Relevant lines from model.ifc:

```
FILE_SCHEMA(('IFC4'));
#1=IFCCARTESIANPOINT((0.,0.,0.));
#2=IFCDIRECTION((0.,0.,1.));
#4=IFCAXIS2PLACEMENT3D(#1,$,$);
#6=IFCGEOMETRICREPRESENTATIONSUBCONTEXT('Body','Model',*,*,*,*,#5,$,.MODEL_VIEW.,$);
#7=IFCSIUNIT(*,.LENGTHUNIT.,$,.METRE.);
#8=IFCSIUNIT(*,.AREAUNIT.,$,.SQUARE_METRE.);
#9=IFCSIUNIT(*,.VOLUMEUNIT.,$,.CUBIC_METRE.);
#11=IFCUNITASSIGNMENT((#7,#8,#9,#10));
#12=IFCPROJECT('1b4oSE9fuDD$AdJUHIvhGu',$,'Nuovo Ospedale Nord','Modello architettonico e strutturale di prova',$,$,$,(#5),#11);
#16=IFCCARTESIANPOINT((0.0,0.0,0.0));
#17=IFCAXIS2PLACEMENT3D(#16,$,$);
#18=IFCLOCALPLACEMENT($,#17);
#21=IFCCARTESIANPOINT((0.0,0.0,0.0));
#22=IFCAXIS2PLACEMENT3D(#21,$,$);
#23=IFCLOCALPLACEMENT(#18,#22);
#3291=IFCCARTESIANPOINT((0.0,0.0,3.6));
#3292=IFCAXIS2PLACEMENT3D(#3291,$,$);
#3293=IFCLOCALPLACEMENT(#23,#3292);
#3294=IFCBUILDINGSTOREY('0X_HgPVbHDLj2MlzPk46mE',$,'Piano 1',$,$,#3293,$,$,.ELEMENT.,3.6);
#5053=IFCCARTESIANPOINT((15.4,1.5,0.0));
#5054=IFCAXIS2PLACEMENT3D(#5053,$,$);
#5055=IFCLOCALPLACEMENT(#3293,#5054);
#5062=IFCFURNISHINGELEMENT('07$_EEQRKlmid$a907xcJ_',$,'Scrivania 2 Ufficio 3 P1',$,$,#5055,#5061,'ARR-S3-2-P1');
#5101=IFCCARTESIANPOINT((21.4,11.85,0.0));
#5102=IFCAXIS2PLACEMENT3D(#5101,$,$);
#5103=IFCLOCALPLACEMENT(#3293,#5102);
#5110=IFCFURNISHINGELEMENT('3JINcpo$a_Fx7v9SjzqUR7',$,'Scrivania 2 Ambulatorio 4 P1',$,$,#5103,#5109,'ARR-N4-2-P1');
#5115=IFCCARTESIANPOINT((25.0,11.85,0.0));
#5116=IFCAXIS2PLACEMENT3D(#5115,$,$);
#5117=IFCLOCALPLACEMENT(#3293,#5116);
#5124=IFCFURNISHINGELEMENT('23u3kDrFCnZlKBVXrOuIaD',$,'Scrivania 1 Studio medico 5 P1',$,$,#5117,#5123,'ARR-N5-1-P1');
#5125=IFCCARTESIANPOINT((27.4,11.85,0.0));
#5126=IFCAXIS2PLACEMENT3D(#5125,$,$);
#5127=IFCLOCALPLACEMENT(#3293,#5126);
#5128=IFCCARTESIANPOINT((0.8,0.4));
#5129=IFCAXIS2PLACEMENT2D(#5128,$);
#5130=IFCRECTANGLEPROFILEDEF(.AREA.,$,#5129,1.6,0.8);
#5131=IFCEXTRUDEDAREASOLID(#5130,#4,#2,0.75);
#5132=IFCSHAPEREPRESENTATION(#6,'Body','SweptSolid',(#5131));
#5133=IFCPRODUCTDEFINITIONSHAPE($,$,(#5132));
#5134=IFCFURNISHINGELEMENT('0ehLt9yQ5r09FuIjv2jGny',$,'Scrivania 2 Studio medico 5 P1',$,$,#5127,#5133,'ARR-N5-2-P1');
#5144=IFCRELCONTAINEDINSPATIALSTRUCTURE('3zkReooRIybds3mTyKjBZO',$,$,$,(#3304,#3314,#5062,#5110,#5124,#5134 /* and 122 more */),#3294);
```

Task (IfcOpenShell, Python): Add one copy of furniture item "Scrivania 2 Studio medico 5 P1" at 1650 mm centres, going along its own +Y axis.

```python
import ifcopenshell
import ifcopenshell.api.geometry
import ifcopenshell.api.root
import ifcopenshell.util.element
import ifcopenshell.util.placement
import ifcopenshell.util.unit

model = ifcopenshell.open("model.ifc")
unit_scale = ifcopenshell.util.unit.calculate_unit_scale(model)

source = model.by_guid("0ehLt9yQ5r09FuIjv2jGny")
base = ifcopenshell.util.placement.get_local_placement(source.ObjectPlacement)
step = base[:3, 1] * 1.65 / unit_scale

for i in range(1, 2):
    copy = ifcopenshell.api.root.copy_class(model, product=source)
    copy.Representation = ifcopenshell.util.element.copy_deep(
        model, source.Representation, exclude=["IfcGeometricRepresentationContext", "IfcRepresentationMap"]
    )
    copy.Tag = None
    matrix = base.copy()
    matrix[:3, 3] += i * step
    print("added at", matrix[:3, 3].round(3) + 0.0)
    ifcopenshell.api.geometry.edit_object_placement(model, product=copy, matrix=matrix, is_si=False)

model.write("model_edited.ifc")
```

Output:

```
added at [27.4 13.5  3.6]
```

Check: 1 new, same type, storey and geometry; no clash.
